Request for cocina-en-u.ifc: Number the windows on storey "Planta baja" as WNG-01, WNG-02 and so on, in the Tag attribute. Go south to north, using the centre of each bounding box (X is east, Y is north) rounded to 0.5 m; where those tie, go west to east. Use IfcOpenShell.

First a look at what the model holds.

```python
import ifcopenshell
import ifcopenshell.util.element
import ifcopenshell.util.placement

model = ifcopenshell.open("cocina-en-u.ifc")
print(model.schema)
storey = next(s for s in model.by_type("IfcBuildingStorey") if s.Name == "Planta baja")
windows = [e for e in ifcopenshell.util.element.get_decomposition(storey) if e.is_a("IfcWindow")]
for e in sorted(windows, key=lambda e: e.id()):
    origin = ifcopenshell.util.placement.get_local_placement(e.ObjectPlacement)[:3, 3]
    print(e.id(), e.Tag, e.Name, origin.round(2) + 0.0, sep=" | ")
```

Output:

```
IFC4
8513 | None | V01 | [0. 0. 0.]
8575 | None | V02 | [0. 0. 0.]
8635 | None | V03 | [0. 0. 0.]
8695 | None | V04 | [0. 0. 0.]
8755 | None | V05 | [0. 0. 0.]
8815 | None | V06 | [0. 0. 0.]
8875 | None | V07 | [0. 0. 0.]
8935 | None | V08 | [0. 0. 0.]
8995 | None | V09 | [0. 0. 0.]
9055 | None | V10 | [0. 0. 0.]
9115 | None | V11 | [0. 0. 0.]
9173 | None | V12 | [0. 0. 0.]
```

```python
import ifcopenshell
import ifcopenshell.geom
import ifcopenshell.util.element
import ifcopenshell.util.shape

model = ifcopenshell.open("cocina-en-u.ifc")
settings = ifcopenshell.geom.settings()
settings.set("use-world-coords", True)


def centre(element):
    shape = ifcopenshell.geom.create_shape(settings, element)
    return ifcopenshell.util.shape.get_bbox_centroid(shape.geometry)


storey = next(s for s in model.by_type("IfcBuildingStorey") if s.Name == "Planta baja")
windows = [e for e in ifcopenshell.util.element.get_decomposition(storey) if e.is_a("IfcWindow")]

# Insertion points can sit at a corner or the storey origin, so sort by the geometry (in metres).
centres = {e: centre(e) for e in windows}
windows.sort(key=lambda e: (round(centres[e][1] / 0.5), centres[e][0]))

for i, e in enumerate(windows, start=1):
    number = f"WNG-{i:02d}"
    e.Tag = number
    print(e.id(), number)

model.write("cocina-en-u-out.ifc")
```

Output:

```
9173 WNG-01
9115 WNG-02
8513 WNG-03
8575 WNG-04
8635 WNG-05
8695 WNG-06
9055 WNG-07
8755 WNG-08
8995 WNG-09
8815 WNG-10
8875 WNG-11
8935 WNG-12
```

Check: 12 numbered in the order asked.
